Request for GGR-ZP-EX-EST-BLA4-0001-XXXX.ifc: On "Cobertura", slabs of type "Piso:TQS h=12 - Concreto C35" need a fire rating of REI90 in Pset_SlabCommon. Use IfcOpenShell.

First a look at what the model holds.

```python
import ifcopenshell
import ifcopenshell.util.element

model = ifcopenshell.open("GGR-ZP-EX-EST-BLA4-0001-XXXX.ifc")
print(model.schema)
storey = next(s for s in model.by_type("IfcBuildingStorey") if s.Name == "Cobertura")
slabs = [e for e in ifcopenshell.util.element.get_decomposition(storey) if e.is_a("IfcSlab")]
seen = {}
for e in slabs:
    element_type = ifcopenshell.util.element.get_type(e)
    key = (element_type.Name if element_type != e and element_type else None, ifcopenshell.util.element.get_pset(e, "Pset_SlabCommon", "FireRating"))
    seen[key] = seen.get(key, 0) + 1
for (name, value), count in sorted(seen.items(), key=str):
    print(count, "x", name, "|", value)
```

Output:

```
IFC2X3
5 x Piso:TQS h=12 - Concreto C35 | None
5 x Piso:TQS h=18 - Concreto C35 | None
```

```python
import ifcopenshell
import ifcopenshell.api.pset
import ifcopenshell.util.element

model = ifcopenshell.open("GGR-ZP-EX-EST-BLA4-0001-XXXX.ifc")

storey = next(s for s in model.by_type("IfcBuildingStorey") if s.Name == "Cobertura")
slabs = [e for e in ifcopenshell.util.element.get_decomposition(storey) if e.is_a("IfcSlab")]

count = 0
for e in slabs:
    element_type = ifcopenshell.util.element.get_type(e)
    if element_type in (None, e) or element_type.Name != "Piso:TQS h=12 - Concreto C35":
        continue
    # add_pset returns the element's existing set when there is one.
    pset = ifcopenshell.api.pset.add_pset(model, product=e, name="Pset_SlabCommon")
    ifcopenshell.api.pset.edit_pset(model, pset=pset, properties={"FireRating": "REI90"})
    count += 1

print(count, "slabs updated")

model.write("GGR-ZP-EX-EST-BLA4-0001-XXXX_edited.ifc")
```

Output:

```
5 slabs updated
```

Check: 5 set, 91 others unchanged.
